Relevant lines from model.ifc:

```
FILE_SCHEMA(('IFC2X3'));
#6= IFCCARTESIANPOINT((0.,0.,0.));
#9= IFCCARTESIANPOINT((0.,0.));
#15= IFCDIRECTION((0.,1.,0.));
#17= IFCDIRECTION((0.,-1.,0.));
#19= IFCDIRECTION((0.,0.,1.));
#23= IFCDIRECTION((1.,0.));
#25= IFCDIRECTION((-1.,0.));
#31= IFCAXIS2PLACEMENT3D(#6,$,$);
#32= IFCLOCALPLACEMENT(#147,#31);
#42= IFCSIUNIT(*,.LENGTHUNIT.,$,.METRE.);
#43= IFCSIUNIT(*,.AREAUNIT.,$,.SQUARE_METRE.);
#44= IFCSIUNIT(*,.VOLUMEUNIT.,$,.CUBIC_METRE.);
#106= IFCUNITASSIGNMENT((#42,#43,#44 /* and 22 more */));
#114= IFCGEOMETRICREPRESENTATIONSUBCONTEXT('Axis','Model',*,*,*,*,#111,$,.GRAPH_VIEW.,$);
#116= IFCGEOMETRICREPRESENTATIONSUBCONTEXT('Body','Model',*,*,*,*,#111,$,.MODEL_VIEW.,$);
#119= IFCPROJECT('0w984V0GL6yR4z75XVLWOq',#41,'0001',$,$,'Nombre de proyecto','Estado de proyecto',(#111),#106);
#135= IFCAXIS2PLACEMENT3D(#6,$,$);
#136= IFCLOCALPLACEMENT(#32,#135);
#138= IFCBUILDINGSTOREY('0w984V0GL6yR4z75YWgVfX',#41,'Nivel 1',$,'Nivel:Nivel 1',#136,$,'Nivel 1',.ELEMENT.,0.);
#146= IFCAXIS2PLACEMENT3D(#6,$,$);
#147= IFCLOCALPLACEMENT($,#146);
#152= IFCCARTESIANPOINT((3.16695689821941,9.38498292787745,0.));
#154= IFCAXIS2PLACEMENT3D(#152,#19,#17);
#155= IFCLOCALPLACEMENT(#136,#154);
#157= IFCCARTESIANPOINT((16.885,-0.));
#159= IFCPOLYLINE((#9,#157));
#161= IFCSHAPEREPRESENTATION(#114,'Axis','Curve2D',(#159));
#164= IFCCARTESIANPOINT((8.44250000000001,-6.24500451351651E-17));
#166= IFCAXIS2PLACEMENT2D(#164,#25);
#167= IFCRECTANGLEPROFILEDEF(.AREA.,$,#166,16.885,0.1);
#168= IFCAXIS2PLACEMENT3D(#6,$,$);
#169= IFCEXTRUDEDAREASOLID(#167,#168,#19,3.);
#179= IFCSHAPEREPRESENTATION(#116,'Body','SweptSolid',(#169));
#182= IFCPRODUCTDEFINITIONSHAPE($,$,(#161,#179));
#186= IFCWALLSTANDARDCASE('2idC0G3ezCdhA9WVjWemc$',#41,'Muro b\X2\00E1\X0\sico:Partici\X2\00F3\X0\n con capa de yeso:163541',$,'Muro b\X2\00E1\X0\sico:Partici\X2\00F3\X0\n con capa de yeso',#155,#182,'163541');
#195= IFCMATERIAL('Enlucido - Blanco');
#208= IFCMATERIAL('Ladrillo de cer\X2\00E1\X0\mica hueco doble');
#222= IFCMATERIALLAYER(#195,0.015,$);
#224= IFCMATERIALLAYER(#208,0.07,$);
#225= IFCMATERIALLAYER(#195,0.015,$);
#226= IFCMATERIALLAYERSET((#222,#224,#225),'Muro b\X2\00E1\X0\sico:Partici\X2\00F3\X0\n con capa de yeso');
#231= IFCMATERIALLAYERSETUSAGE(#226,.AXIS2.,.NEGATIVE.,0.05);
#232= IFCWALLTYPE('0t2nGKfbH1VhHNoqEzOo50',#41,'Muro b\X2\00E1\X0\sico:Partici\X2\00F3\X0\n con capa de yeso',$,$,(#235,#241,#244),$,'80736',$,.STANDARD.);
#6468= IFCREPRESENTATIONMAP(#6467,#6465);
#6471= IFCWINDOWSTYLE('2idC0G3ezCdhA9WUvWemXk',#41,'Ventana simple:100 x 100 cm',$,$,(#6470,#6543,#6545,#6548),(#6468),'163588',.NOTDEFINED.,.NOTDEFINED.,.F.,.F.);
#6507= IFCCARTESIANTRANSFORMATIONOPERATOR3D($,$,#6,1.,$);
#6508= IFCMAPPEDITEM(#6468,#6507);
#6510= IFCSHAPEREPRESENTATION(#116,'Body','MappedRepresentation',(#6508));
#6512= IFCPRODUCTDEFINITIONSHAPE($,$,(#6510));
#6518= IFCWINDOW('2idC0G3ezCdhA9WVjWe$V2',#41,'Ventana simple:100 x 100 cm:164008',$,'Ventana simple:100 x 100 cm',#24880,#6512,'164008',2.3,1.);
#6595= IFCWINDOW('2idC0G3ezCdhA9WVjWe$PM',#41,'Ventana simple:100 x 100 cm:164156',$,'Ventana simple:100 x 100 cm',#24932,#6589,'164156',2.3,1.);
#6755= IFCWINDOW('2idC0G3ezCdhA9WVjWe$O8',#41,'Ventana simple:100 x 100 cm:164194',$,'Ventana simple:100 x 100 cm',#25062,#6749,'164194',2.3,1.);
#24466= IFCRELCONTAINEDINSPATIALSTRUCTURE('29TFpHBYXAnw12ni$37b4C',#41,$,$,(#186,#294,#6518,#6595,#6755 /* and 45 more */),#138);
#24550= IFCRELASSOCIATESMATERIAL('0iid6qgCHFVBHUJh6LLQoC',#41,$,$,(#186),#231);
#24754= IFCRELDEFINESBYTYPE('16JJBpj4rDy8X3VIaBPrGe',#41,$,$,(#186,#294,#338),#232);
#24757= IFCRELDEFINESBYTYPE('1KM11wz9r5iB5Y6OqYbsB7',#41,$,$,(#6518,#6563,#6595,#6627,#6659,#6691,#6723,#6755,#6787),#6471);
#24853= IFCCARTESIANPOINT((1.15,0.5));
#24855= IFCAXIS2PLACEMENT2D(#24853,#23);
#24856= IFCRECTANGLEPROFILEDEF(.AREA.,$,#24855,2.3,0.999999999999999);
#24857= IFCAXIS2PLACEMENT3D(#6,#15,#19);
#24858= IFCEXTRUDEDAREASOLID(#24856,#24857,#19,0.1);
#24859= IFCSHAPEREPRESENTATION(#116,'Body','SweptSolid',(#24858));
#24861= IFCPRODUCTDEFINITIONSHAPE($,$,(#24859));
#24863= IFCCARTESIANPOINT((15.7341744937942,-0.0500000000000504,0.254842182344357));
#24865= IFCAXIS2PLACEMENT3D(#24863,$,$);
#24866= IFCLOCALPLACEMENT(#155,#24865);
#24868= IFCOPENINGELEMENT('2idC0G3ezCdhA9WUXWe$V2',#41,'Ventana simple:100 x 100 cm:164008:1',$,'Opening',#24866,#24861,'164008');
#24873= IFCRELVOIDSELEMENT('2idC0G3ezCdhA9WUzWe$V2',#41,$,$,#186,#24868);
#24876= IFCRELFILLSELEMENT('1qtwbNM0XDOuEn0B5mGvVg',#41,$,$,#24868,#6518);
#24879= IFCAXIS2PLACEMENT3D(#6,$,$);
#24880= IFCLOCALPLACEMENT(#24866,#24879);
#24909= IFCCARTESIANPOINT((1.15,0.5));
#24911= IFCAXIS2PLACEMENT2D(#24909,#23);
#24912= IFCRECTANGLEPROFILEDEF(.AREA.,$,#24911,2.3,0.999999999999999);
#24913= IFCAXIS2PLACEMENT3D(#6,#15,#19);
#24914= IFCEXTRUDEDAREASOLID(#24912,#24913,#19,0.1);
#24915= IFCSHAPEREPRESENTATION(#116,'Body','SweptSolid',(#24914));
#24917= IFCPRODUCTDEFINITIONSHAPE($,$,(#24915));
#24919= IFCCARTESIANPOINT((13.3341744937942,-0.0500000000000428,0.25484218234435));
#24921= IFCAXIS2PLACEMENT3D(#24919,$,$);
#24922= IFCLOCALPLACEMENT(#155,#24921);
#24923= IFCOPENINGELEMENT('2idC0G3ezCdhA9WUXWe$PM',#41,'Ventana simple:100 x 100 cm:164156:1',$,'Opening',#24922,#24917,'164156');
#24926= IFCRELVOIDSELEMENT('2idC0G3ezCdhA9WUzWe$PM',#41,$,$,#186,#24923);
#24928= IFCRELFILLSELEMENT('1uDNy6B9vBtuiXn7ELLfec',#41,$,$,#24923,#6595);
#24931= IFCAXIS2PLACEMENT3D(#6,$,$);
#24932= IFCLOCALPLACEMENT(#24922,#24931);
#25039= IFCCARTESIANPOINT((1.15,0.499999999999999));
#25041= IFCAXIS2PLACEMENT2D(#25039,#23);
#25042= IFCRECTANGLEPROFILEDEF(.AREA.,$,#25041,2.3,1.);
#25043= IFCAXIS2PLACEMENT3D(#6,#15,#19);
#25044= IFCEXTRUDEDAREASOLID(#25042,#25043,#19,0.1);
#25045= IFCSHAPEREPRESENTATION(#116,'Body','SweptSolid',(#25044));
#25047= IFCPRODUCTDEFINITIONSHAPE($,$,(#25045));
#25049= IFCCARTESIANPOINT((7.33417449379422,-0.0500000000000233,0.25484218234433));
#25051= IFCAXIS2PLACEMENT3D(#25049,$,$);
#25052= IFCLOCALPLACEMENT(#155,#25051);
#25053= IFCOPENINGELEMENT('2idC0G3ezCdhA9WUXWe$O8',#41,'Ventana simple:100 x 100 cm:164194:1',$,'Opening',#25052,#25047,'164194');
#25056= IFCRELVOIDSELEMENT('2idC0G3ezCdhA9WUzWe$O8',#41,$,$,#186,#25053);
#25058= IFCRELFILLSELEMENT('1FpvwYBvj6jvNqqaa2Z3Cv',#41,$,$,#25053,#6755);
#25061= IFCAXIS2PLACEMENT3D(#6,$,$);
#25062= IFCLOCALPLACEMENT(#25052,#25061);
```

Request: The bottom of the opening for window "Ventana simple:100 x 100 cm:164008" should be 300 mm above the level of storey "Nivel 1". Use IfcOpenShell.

```python
import numpy as np
import ifcopenshell
import ifcopenshell.api.geometry
import ifcopenshell.geom
import ifcopenshell.util.element
import ifcopenshell.util.placement
import ifcopenshell.util.shape
import ifcopenshell.util.unit

model = ifcopenshell.open("model.ifc")
unit_scale = ifcopenshell.util.unit.calculate_unit_scale(model)

window = model.by_guid("2idC0G3ezCdhA9WVjWe$V2")
opening = window.FillsVoids[0].RelatingOpeningElement
storey = ifcopenshell.util.element.get_container(window, ifc_class="IfcBuildingStorey")
level = ifcopenshell.util.placement.get_local_placement(storey.ObjectPlacement)[2, 3]

# The opening's origin need not be at the sill, so measure its lowest point.
shape = ifcopenshell.geom.create_shape(ifcopenshell.geom.settings(), opening)
bottom = ifcopenshell.util.shape.get_shape_bottom_elevation(shape, shape.geometry) / unit_scale
dz = level + 0.3 / unit_scale - bottom

shift = np.array([0.0, 0.0, dz])
# The window is placed relative to its opening, so it follows when the opening moves.
matrix = ifcopenshell.util.placement.get_local_placement(opening.ObjectPlacement)
matrix[:3, 3] += shift
ifcopenshell.api.geometry.edit_object_placement(
    model, product=opening, matrix=matrix, is_si=False, should_transform_children=True
)

print(f"moved by {dz * unit_scale:+.3f} m")

model.write("model_rev.ifc")
```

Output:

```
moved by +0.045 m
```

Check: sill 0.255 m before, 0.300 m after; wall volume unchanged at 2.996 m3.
